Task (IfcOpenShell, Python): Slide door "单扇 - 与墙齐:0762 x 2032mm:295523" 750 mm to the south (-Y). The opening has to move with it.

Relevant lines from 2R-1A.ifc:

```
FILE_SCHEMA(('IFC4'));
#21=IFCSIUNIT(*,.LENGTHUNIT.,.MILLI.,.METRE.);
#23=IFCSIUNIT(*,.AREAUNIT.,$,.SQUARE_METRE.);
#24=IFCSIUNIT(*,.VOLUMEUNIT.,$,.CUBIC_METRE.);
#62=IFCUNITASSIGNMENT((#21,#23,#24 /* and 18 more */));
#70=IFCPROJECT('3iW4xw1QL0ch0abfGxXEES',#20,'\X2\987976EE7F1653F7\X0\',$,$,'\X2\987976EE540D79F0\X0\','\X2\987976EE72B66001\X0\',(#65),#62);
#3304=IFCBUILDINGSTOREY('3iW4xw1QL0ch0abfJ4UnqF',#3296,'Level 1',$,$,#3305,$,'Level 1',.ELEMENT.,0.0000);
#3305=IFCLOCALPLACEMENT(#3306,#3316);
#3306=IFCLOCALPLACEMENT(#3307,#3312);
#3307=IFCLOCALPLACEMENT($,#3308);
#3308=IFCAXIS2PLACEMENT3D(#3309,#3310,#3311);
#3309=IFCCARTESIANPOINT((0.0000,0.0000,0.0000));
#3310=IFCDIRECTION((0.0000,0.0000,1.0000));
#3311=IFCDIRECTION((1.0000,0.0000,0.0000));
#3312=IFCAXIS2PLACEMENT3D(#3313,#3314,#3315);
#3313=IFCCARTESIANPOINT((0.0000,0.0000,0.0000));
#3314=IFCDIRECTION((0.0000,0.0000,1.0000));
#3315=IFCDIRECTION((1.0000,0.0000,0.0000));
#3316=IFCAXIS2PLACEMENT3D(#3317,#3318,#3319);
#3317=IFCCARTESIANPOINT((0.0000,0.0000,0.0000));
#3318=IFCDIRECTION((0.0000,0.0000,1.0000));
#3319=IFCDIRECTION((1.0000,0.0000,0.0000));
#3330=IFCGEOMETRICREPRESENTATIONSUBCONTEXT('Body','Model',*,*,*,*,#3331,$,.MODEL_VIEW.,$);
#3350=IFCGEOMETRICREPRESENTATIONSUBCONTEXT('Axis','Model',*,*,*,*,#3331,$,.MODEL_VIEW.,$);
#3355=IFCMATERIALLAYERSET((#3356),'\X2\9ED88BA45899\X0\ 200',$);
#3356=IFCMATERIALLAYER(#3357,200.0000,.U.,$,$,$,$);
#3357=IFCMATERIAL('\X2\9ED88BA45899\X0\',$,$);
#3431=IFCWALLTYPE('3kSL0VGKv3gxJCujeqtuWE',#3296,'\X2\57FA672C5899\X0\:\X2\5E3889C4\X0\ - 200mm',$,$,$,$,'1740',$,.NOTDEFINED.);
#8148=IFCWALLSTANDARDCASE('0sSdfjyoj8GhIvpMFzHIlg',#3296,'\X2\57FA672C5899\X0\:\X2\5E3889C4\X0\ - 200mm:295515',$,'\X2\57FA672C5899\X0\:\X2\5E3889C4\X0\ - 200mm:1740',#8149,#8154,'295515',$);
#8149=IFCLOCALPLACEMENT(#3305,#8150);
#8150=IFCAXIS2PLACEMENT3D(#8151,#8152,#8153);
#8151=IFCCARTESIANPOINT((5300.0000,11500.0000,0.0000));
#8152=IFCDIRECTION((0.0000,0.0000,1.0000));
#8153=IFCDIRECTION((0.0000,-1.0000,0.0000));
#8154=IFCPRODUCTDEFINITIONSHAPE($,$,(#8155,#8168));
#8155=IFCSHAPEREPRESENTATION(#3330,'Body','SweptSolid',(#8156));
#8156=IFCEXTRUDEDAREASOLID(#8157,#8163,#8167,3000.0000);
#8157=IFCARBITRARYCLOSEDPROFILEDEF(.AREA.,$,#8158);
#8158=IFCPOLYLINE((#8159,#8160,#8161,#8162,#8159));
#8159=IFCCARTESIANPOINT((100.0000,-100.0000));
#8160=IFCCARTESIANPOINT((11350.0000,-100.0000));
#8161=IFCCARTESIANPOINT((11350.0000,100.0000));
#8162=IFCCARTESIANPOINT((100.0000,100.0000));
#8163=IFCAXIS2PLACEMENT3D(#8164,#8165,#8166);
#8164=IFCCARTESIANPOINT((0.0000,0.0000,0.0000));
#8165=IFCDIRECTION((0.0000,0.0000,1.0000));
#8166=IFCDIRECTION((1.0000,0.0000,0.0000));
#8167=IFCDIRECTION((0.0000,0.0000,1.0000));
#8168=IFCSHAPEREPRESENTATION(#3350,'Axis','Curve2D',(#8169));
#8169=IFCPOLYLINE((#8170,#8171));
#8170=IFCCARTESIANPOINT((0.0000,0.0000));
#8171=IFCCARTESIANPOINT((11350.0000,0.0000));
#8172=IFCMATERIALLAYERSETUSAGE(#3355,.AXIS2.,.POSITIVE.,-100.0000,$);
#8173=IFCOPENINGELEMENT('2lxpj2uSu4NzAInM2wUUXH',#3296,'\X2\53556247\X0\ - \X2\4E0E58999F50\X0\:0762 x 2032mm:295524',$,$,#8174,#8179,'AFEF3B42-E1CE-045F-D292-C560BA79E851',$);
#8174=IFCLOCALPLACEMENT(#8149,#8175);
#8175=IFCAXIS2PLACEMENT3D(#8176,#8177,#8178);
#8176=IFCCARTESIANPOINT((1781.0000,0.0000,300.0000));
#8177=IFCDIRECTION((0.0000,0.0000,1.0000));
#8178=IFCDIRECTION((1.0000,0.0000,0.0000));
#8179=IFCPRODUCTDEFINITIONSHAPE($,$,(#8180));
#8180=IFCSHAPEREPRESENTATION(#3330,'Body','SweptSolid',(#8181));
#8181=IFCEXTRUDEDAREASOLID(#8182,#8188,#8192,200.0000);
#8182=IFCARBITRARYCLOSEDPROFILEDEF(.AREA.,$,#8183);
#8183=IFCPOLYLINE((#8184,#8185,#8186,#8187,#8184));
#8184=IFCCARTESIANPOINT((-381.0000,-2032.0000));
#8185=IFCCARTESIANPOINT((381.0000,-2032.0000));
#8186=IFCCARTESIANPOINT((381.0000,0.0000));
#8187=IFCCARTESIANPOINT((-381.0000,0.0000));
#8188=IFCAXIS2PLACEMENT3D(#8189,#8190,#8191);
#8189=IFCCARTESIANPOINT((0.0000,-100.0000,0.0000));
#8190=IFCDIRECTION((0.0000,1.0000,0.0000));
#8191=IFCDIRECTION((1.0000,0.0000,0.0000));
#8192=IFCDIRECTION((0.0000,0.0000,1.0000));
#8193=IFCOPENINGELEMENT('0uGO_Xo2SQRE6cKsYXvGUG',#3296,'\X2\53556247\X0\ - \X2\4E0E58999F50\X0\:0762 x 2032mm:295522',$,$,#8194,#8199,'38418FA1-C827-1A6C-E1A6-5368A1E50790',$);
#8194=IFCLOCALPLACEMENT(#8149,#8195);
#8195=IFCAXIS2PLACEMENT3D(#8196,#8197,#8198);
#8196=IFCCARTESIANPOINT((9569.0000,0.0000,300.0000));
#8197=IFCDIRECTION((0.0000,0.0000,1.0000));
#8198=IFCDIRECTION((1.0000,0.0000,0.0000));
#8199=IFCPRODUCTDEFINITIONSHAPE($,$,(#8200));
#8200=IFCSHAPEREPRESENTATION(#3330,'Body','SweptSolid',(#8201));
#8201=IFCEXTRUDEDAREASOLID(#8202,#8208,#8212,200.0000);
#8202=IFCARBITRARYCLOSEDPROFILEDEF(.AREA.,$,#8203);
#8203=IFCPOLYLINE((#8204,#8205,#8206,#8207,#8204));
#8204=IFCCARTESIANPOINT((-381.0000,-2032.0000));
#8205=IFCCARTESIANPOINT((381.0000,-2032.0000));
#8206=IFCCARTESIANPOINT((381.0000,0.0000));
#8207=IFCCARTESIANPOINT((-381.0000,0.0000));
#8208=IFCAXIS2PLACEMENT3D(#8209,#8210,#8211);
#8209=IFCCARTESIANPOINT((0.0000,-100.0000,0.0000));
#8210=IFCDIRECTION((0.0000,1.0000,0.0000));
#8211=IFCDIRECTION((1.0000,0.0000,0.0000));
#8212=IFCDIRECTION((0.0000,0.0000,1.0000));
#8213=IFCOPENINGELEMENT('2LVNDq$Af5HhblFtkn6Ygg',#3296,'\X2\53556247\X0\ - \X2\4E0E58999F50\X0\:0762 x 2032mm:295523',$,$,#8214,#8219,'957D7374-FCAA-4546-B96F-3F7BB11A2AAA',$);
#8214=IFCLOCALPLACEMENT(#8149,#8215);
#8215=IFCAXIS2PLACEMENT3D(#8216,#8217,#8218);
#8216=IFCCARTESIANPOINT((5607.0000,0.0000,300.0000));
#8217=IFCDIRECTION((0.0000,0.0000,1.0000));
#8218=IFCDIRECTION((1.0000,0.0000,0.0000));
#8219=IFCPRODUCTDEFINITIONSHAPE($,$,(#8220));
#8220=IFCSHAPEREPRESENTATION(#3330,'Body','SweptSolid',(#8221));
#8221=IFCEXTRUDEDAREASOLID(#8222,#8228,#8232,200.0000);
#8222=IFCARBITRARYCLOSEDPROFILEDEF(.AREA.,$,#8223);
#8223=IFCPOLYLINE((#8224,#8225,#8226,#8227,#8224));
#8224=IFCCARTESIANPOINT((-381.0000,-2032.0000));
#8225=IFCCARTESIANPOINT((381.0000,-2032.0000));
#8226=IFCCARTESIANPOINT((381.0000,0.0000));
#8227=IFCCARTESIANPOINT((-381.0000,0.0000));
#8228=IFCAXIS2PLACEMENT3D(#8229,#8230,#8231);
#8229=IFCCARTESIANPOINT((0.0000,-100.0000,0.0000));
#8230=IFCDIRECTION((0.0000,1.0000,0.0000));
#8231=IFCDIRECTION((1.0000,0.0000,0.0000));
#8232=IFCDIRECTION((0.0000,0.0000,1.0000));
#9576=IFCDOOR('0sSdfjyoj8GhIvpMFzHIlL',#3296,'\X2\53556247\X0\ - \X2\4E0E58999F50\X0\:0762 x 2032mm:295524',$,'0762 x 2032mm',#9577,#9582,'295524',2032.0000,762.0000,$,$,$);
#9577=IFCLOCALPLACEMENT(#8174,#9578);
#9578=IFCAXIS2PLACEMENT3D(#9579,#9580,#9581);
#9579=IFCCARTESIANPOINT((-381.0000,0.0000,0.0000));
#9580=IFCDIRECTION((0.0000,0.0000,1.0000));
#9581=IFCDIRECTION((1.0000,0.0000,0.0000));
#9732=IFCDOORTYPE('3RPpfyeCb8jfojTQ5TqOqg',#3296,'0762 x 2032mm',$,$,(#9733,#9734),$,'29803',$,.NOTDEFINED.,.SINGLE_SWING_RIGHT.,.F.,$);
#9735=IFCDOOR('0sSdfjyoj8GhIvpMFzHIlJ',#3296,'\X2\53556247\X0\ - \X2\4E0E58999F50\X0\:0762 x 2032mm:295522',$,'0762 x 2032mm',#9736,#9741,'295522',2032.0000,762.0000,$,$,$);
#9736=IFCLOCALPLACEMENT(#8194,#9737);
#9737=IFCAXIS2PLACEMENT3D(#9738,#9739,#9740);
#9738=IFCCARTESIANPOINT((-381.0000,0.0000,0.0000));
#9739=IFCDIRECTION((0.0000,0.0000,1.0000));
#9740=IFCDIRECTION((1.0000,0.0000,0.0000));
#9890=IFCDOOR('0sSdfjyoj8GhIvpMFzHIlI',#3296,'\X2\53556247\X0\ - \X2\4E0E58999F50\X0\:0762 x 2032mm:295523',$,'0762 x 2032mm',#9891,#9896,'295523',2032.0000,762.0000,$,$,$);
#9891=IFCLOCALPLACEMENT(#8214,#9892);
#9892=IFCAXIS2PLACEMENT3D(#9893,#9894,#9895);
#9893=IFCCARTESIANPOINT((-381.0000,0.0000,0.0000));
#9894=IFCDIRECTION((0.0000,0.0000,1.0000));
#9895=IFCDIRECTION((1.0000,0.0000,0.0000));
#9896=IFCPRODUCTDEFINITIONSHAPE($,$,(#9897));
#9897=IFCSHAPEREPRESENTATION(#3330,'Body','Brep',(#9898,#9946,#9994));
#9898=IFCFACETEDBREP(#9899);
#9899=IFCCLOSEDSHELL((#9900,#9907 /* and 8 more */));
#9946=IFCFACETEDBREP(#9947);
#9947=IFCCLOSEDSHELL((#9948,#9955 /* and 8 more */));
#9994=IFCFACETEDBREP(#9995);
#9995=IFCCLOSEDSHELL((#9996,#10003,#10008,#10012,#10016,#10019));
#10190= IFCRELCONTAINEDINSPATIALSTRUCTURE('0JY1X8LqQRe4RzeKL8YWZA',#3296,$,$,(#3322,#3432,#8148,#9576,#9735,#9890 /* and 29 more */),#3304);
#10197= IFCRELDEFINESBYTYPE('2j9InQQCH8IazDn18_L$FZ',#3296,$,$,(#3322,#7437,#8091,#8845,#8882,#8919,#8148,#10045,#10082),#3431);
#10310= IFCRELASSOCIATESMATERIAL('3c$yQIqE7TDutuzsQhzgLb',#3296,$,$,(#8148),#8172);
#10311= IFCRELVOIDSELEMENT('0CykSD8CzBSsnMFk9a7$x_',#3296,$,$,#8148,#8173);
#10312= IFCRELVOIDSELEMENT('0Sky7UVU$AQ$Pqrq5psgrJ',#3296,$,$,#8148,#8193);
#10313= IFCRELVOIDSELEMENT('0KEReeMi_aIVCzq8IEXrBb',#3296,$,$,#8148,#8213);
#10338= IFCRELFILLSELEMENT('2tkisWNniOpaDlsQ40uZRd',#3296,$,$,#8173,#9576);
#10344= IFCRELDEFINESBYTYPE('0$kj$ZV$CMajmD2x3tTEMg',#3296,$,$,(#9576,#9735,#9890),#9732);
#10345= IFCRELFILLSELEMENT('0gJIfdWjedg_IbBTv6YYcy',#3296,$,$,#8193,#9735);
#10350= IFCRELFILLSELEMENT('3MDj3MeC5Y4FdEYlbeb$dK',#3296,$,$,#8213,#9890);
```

```python
import ifcopenshell
import ifcopenshell.api.geometry
import ifcopenshell.util.placement
import ifcopenshell.util.unit

model = ifcopenshell.open("2R-1A.ifc")
unit_scale = ifcopenshell.util.unit.calculate_unit_scale(model)

door = model.by_guid("0sSdfjyoj8GhIvpMFzHIlI")
opening = door.FillsVoids[0].RelatingOpeningElement
wall = opening.VoidsElements[0].RelatingBuildingElement

wall_matrix = ifcopenshell.util.placement.get_local_placement(wall.ObjectPlacement)
shift = wall_matrix[:3, 0] * 0.75 / unit_scale
before = ifcopenshell.util.placement.get_local_placement(door.ObjectPlacement)[:3, 3].copy()

# The door is placed relative to its opening, so it follows when the opening moves.
matrix = ifcopenshell.util.placement.get_local_placement(opening.ObjectPlacement)
matrix[:3, 3] += shift
ifcopenshell.api.geometry.edit_object_placement(
    model, product=opening, matrix=matrix, is_si=False, should_transform_children=True
)

after = ifcopenshell.util.placement.get_local_placement(door.ObjectPlacement)[:3, 3]
print("door moved by", (after - before).round(3) + 0.0)

model.write("2R-1A_edited.ifc")
```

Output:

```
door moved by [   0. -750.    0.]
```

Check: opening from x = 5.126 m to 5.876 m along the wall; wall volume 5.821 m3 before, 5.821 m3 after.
